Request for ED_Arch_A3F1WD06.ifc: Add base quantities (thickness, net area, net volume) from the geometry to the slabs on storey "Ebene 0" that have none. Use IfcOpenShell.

First a look at what the model holds.

```python
import ifcopenshell
import ifcopenshell.util.element
import ifcopenshell.util.unit

model = ifcopenshell.open("ED_Arch_A3F1WD06.ifc")
print(model.schema)
for unit_type in ("LENGTHUNIT", "AREAUNIT", "VOLUMEUNIT"):
    print(unit_type, ifcopenshell.util.unit.calculate_unit_scale(model, unit_type))
storey = next(s for s in model.by_type("IfcBuildingStorey") if s.Name == "Ebene 0")
slabs = [e for e in ifcopenshell.util.element.get_decomposition(storey) if e.is_a("IfcSlab")]
for e in sorted(slabs, key=lambda e: e.id()):
    print(e.id(), e.is_a(), e.Name, list(ifcopenshell.util.element.get_psets(e, qtos_only=True)), sep=" | ")
```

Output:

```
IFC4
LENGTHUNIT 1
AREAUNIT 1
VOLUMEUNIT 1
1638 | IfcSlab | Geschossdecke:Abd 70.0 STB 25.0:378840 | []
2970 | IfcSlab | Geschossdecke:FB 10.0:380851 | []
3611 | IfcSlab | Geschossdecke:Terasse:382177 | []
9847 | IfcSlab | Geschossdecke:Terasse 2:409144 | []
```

```python
import ifcopenshell
import ifcopenshell.api.pset
import ifcopenshell.geom
import ifcopenshell.util.element
import ifcopenshell.util.shape
import ifcopenshell.util.unit

model = ifcopenshell.open("ED_Arch_A3F1WD06.ifc")
unit_scale = ifcopenshell.util.unit.calculate_unit_scale(model)
area_scale = ifcopenshell.util.unit.calculate_unit_scale(model, "AREAUNIT")
volume_scale = ifcopenshell.util.unit.calculate_unit_scale(model, "VOLUMEUNIT")
settings = ifcopenshell.geom.settings()

storey = next(s for s in model.by_type("IfcBuildingStorey") if s.Name == "Ebene 0")
slabs = [e for e in ifcopenshell.util.element.get_decomposition(storey) if e.is_a("IfcSlab")]

for e in sorted(slabs, key=lambda e: e.id()):
    if ifcopenshell.util.element.get_psets(e, qtos_only=True, should_inherit=False):
        continue
    # Geometry comes back in metres, in the element's own axes.
    shape = ifcopenshell.geom.create_shape(settings, e)
    values = {
        "Width": ifcopenshell.util.shape.get_z(shape.geometry) / unit_scale,
        "NetArea": ifcopenshell.util.shape.get_footprint_area(shape.geometry) / area_scale,
        "NetVolume": ifcopenshell.util.shape.get_volume(shape.geometry) / volume_scale,
    }
    qto = ifcopenshell.api.pset.add_qto(model, product=e, name="Qto_SlabBaseQuantities")
    ifcopenshell.api.pset.edit_qto(model, qto=qto, properties=values)
    print(e.id(), {k: round(v, 3) for k, v in values.items()})

model.write("ED_Arch_A3F1WD06_edited.ifc")
```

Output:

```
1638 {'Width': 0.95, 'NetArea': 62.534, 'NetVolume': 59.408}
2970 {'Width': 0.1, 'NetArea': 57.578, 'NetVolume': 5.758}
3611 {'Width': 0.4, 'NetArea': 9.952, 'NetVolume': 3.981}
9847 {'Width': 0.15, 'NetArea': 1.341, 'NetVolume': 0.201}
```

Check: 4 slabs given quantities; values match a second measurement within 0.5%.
